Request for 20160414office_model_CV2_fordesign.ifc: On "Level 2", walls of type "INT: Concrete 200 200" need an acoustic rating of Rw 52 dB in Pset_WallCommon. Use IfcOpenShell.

First a look at what the model holds.

```python
import ifcopenshell
import ifcopenshell.util.element

model = ifcopenshell.open("20160414office_model_CV2_fordesign.ifc")
print(model.schema)
storey = next(s for s in model.by_type("IfcBuildingStorey") if s.Name == "Level 2")
walls = [e for e in ifcopenshell.util.element.get_decomposition(storey) if e.is_a("IfcWall")]
seen = {}
for e in walls:
    element_type = ifcopenshell.util.element.get_type(e)
    key = (element_type.Name if element_type != e and element_type else None, ifcopenshell.util.element.get_pset(e, "Pset_WallCommon", "AcousticRating"))
    seen[key] = seen.get(key, 0) + 1
for (name, value), count in sorted(seen.items(), key=str):
    print(count, "x", name, "|", value)
```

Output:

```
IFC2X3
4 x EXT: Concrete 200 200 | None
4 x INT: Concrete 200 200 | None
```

```python
import ifcopenshell
import ifcopenshell.api.pset
import ifcopenshell.util.element

model = ifcopenshell.open("20160414office_model_CV2_fordesign.ifc")

storey = next(s for s in model.by_type("IfcBuildingStorey") if s.Name == "Level 2")
walls = [e for e in ifcopenshell.util.element.get_decomposition(storey) if e.is_a("IfcWall")]

count = 0
for e in walls:
    element_type = ifcopenshell.util.element.get_type(e)
    if element_type in (None, e) or element_type.Name != "INT: Concrete 200 200":
        continue
    # add_pset returns the element's existing set when there is one.
    pset = ifcopenshell.api.pset.add_pset(model, product=e, name="Pset_WallCommon")
    ifcopenshell.api.pset.edit_pset(model, pset=pset, properties={"AcousticRating": "Rw 52 dB"})
    count += 1

print(count, "walls updated")

model.write("20160414office_model_CV2_fordesign_edited.ifc")
```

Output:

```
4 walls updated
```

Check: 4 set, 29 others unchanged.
